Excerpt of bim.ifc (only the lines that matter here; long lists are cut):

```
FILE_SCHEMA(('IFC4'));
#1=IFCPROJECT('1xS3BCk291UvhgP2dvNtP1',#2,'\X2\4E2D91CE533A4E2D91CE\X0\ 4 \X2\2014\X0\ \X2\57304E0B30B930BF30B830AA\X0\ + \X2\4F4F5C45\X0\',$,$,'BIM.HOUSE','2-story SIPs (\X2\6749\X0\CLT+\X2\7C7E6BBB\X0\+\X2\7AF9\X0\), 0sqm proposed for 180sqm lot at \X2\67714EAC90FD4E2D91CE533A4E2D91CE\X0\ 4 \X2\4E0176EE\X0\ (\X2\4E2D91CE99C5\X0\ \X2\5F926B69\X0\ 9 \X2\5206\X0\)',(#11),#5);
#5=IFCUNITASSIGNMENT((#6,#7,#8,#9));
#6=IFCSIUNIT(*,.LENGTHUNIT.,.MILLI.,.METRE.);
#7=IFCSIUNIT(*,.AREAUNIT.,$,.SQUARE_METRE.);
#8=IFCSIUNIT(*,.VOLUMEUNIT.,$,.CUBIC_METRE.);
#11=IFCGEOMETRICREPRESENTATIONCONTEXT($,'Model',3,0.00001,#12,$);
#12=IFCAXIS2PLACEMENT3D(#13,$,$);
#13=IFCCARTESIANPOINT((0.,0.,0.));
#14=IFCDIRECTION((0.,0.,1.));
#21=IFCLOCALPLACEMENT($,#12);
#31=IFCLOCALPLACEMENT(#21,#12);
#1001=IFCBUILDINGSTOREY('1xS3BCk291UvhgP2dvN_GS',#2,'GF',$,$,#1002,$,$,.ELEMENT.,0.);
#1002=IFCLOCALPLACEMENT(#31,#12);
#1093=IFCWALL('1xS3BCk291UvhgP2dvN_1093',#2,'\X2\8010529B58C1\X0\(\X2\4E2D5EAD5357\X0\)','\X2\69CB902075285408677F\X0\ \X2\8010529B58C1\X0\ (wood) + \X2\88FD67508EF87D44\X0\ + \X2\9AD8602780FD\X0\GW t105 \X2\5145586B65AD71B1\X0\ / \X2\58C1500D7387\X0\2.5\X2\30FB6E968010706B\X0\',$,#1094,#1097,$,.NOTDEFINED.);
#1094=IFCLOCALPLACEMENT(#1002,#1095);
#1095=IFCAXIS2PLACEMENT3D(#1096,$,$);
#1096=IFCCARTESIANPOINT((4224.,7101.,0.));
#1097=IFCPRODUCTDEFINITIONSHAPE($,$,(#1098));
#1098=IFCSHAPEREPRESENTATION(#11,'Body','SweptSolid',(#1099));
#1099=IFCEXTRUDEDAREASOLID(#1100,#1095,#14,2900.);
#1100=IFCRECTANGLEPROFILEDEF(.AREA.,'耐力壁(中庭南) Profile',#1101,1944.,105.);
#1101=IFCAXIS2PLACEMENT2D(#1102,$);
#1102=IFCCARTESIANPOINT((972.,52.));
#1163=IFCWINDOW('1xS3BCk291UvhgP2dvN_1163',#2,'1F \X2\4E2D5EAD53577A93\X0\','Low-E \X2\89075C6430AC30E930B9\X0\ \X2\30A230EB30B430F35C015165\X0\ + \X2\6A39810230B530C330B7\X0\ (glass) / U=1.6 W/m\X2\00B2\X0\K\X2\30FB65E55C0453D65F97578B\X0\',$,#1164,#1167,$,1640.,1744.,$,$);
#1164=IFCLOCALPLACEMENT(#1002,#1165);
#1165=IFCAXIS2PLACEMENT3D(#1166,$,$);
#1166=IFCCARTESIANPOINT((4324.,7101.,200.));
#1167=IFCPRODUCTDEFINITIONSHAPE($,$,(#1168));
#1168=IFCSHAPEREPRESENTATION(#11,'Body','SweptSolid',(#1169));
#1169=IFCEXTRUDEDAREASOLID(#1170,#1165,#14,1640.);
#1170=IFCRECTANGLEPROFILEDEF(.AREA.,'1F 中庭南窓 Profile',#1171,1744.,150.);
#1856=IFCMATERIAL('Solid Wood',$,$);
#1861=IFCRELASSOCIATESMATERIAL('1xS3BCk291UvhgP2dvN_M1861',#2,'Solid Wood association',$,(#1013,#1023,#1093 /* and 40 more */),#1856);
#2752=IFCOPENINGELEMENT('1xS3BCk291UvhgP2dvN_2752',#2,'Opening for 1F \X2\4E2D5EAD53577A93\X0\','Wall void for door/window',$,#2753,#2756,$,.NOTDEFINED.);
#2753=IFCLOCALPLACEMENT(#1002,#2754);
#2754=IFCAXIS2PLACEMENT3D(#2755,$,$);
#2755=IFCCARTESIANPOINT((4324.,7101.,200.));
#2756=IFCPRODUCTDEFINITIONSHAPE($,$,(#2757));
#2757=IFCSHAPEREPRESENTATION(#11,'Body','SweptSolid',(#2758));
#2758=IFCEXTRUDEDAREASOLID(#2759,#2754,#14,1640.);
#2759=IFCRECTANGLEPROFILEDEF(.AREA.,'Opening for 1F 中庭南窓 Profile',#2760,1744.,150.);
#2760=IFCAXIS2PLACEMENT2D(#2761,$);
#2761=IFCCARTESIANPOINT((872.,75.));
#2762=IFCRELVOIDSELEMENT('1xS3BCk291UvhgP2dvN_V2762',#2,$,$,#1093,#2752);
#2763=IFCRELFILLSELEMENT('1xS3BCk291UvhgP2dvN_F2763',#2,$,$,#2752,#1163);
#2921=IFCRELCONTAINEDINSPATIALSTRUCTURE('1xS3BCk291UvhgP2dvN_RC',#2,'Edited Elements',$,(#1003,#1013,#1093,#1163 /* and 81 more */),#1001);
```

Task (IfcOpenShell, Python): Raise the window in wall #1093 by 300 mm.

```python
import numpy as np
import ifcopenshell
import ifcopenshell.api.geometry
import ifcopenshell.util.placement
import ifcopenshell.util.unit

model = ifcopenshell.open("bim.ifc")
unit_scale = ifcopenshell.util.unit.calculate_unit_scale(model)

window = model.by_id(1163)
opening = window.FillsVoids[0].RelatingOpeningElement
dz = 300.0

shift = np.array([0.0, 0.0, dz])
# The window is not placed relative to its opening, so move both.
for product in (opening, window):
    matrix = ifcopenshell.util.placement.get_local_placement(product.ObjectPlacement)
    matrix[:3, 3] += shift
    ifcopenshell.api.geometry.edit_object_placement(model, product=product, matrix=matrix, is_si=False)

print(f"moved by {dz * unit_scale:+.3f} m")

model.write("bim_rev.ifc")
```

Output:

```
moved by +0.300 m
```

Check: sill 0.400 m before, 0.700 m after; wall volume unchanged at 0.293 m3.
